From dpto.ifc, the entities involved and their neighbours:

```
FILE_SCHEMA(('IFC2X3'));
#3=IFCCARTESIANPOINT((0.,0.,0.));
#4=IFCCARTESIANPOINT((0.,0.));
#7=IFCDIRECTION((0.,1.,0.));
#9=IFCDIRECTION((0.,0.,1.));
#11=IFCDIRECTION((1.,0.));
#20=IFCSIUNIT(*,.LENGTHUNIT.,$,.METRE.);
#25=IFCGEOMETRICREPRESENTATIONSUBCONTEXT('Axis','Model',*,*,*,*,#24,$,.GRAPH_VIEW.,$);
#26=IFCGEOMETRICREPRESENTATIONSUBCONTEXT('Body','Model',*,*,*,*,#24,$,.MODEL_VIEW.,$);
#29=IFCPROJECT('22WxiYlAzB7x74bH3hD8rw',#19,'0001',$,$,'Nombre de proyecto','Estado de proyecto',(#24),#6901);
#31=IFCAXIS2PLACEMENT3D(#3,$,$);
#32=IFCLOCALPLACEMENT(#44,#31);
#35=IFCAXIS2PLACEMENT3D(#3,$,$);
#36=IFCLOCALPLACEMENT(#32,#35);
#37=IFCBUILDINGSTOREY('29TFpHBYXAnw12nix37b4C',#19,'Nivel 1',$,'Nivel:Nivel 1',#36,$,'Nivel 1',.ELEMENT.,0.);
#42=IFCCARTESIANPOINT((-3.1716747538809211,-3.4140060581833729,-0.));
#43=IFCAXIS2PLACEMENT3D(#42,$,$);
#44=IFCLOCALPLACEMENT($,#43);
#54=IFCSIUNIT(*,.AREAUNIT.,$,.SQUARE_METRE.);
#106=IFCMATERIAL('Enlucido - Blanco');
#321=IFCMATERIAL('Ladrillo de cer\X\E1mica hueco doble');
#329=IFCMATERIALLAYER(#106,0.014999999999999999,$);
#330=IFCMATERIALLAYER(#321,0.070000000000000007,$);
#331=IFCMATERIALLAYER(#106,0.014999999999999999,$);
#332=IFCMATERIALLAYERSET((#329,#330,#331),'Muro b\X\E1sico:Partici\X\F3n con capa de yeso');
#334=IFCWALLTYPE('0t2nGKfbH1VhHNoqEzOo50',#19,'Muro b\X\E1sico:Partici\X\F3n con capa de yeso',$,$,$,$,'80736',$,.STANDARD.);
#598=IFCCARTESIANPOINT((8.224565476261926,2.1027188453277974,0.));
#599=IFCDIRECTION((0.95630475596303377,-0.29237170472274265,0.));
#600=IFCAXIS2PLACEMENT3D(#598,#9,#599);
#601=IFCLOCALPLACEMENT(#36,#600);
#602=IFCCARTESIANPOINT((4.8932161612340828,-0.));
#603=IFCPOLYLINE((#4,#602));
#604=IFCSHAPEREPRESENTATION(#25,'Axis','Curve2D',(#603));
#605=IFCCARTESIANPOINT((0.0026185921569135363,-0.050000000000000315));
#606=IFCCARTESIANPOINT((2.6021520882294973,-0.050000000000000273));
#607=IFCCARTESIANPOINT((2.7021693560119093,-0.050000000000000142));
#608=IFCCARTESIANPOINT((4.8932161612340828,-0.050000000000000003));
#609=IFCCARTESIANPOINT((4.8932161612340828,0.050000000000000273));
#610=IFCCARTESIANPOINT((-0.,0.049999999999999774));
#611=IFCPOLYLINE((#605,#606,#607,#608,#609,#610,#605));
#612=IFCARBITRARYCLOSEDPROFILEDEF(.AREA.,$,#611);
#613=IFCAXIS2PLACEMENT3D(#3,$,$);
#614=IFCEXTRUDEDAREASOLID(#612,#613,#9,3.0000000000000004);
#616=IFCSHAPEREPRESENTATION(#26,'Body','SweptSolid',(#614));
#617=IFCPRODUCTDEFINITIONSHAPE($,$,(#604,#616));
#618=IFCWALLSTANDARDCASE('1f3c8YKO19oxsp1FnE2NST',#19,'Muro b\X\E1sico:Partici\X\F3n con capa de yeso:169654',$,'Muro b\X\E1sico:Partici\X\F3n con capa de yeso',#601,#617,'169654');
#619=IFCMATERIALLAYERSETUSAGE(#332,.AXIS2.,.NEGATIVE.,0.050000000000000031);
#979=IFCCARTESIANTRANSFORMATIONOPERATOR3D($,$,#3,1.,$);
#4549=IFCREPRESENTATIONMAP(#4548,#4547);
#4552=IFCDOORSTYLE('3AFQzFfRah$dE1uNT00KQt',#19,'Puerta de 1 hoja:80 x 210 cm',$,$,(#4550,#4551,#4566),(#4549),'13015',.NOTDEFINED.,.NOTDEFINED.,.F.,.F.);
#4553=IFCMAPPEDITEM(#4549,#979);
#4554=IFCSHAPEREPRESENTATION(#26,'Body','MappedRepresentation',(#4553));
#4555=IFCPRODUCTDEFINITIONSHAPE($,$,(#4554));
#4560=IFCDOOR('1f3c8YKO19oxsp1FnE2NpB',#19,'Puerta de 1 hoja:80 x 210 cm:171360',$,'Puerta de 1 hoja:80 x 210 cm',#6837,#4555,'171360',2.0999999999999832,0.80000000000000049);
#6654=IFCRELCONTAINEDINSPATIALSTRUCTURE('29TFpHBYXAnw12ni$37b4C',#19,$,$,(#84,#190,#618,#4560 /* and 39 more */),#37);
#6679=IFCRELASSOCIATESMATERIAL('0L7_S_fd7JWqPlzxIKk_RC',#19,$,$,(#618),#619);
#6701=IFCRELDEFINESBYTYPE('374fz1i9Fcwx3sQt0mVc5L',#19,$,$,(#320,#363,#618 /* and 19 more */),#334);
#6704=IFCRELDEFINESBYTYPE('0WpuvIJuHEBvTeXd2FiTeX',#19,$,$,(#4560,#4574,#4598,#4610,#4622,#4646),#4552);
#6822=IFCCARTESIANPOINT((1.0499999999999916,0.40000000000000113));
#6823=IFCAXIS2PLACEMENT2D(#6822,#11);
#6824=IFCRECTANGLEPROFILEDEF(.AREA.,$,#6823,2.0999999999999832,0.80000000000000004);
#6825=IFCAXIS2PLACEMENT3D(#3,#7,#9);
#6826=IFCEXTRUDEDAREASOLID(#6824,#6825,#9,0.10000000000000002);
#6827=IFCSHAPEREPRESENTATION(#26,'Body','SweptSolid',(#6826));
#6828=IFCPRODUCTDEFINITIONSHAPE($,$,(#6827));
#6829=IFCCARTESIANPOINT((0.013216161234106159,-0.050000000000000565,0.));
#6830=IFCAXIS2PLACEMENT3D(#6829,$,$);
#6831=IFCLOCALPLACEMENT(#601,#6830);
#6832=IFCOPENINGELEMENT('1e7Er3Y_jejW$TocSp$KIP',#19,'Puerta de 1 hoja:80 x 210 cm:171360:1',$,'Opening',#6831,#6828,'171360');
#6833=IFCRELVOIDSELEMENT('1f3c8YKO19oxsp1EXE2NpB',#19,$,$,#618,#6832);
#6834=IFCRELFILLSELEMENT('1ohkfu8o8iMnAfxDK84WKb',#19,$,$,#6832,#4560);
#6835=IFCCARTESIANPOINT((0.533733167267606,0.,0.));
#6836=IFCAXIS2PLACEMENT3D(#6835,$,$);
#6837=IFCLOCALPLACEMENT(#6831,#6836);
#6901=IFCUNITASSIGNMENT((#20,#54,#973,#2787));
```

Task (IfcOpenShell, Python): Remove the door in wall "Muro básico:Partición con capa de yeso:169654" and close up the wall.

```python
import ifcopenshell
import ifcopenshell.api.feature
import ifcopenshell.api.root
import ifcopenshell.geom
import ifcopenshell.util.shape

model = ifcopenshell.open("dpto.ifc")
settings = ifcopenshell.geom.settings()


def volume(element):
    """Net volume in cubic metres, openings subtracted."""
    shape = ifcopenshell.geom.create_shape(settings, element)
    return ifcopenshell.util.shape.get_volume(shape.geometry)


door = model.by_guid("1f3c8YKO19oxsp1FnE2NpB")
opening = door.FillsVoids[0].RelatingOpeningElement
wall = opening.VoidsElements[0].RelatingBuildingElement
before = volume(wall)

ifcopenshell.api.root.remove_product(model, product=door)
ifcopenshell.api.feature.remove_feature(model, feature=opening)

after = volume(wall)

print(f"wall volume {before:.3f} -> {after:.3f} m3")

model.write("dpto_rev.ifc")
```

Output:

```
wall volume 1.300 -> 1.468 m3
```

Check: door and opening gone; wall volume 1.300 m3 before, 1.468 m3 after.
